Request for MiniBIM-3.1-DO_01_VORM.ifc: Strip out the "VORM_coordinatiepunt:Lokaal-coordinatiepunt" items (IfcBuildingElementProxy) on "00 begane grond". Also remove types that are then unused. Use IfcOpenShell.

First a look at what the model holds.

```python
import ifcopenshell
import ifcopenshell.util.element

model = ifcopenshell.open("MiniBIM-3.1-DO_01_VORM.ifc")
print(model.schema)
storey = next(s for s in model.by_type("IfcBuildingStorey") if s.Name == "00 begane grond")
proxies = [e for e in ifcopenshell.util.element.get_decomposition(storey) if e.is_a("IfcBuildingElementProxy")]
seen = {}
for e in proxies:
    element_type = ifcopenshell.util.element.get_type(e)
    name = element_type.Name if element_type not in (None, e) else None
    seen[name] = seen.get(name, 0) + 1
for name, count in sorted(seen.items(), key=str):
    print(count, "x", name)
```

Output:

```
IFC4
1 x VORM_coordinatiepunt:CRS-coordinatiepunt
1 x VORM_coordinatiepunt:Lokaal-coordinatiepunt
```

```python
import ifcopenshell
import ifcopenshell.api.root
import ifcopenshell.util.element

model = ifcopenshell.open("MiniBIM-3.1-DO_01_VORM.ifc")

storey = next(s for s in model.by_type("IfcBuildingStorey") if s.Name == "00 begane grond")
proxies = [e for e in ifcopenshell.util.element.get_decomposition(storey) if e.is_a("IfcBuildingElementProxy")]
targets = [e for e in proxies if (t := ifcopenshell.util.element.get_type(e)) not in (None, e) and t.Name == "VORM_coordinatiepunt:Lokaal-coordinatiepunt"]
types = {ifcopenshell.util.element.get_type(e) for e in targets} - {None, *targets}

for e in targets:
    ifcopenshell.api.root.remove_product(model, product=e)
print(len(targets), "removed")

unused = [t for t in types if not ifcopenshell.util.element.get_types(t)]
for t in unused:
    ifcopenshell.api.root.remove_product(model, product=t)
print(len(unused), "unused types removed")

model.write("MiniBIM-3.1-DO_01_VORM_edited.ifc")
```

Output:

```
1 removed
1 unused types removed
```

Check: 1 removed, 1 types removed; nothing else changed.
